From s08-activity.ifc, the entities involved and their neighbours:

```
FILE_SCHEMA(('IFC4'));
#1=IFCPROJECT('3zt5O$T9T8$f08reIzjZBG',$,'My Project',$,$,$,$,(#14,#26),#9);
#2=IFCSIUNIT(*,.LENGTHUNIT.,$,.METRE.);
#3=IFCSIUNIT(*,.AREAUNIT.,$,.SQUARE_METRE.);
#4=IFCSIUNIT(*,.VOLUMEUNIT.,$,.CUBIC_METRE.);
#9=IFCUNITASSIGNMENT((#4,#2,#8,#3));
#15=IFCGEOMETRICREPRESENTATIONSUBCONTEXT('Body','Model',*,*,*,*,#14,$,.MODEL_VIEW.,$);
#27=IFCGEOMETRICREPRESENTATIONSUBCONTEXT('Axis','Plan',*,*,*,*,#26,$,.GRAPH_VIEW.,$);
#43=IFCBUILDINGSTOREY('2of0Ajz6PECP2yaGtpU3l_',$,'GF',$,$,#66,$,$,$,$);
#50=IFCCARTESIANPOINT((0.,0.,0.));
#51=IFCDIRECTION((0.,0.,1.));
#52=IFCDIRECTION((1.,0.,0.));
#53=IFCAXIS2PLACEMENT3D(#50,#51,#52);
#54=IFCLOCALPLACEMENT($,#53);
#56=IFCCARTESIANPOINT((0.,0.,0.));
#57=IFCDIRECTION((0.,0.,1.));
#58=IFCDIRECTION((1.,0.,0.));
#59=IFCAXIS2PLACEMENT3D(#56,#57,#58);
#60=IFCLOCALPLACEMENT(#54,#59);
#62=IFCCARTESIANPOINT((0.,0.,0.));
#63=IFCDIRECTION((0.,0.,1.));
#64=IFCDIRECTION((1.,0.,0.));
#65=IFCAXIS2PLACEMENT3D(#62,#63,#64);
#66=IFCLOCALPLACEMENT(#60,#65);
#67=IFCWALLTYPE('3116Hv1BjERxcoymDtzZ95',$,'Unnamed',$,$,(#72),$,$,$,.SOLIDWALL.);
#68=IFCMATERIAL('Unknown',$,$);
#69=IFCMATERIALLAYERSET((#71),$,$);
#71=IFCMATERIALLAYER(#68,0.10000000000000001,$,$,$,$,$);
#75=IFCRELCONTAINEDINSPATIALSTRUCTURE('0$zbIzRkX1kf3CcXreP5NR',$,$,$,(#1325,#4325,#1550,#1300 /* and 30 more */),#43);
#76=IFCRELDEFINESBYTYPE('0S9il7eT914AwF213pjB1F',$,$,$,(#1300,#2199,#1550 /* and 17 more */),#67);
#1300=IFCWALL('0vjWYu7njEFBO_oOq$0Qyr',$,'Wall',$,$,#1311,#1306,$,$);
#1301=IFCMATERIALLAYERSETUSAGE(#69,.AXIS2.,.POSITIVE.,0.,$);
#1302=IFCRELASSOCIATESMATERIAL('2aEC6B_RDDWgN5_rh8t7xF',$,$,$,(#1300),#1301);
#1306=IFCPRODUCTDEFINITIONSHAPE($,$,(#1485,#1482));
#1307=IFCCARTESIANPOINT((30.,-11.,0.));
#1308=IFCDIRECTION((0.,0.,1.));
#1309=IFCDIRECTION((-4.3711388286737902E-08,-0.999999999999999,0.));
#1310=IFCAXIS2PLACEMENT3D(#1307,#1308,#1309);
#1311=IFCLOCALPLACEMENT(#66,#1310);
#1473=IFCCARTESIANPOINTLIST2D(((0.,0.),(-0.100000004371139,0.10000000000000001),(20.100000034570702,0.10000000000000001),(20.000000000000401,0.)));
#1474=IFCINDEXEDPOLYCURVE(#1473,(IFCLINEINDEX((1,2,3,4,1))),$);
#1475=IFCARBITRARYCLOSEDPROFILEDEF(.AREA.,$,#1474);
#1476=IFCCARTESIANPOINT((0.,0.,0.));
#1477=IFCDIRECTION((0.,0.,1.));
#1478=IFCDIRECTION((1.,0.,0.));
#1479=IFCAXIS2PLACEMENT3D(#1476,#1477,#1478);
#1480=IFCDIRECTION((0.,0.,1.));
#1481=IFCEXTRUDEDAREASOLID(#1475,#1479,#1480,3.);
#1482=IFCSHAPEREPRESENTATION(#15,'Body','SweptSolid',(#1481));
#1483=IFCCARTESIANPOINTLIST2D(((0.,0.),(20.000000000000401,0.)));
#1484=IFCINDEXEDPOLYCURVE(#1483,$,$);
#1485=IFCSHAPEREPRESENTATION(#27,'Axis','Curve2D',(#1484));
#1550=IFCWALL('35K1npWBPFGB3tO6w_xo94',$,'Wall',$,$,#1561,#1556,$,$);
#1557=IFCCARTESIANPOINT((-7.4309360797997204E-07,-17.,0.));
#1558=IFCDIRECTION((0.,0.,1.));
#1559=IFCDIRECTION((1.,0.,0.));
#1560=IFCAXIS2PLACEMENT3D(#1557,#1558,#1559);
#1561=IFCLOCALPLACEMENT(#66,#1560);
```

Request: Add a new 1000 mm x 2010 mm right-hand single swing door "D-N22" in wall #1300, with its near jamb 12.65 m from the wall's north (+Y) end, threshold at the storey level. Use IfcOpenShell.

```python
import numpy as np
import ifcopenshell
import ifcopenshell.api.feature
import ifcopenshell.api.geometry
import ifcopenshell.api.root
import ifcopenshell.api.spatial
import ifcopenshell.geom
import ifcopenshell.util.element
import ifcopenshell.util.placement
import ifcopenshell.util.representation
import ifcopenshell.util.shape
import ifcopenshell.util.unit

model = ifcopenshell.open("s08-activity.ifc")
unit_scale = ifcopenshell.util.unit.calculate_unit_scale(model)
settings = ifcopenshell.geom.settings()


def volume(element):
    """Net volume in cubic metres, openings subtracted."""
    shape = ifcopenshell.geom.create_shape(settings, element)
    return ifcopenshell.util.shape.get_volume(shape.geometry)


wall = model.by_guid("0vjWYu7njEFBO_oOq$0Qyr")
storey = ifcopenshell.util.element.get_container(wall, ifc_class="IfcBuildingStorey")
context = ifcopenshell.util.representation.get_context(model, "Model", "Body", "MODEL_VIEW")
before = volume(wall)

width, height, from_end, sill = 1, 2.01, 12.65, 0.0  # metres

# The wall runs along its own X axis, and the end named is its -X end.
wall_shape = ifcopenshell.geom.create_shape(settings, wall)
x, y, z = ifcopenshell.util.shape.get_vertices(wall_shape.geometry).T
start = x.min() + from_end
face, thickness = float(y.min()), float(y.max() - y.min())
wall_matrix = ifcopenshell.util.placement.get_local_placement(wall.ObjectPlacement)
level = ifcopenshell.util.placement.get_local_placement(storey.ObjectPlacement)[2, 3]


def in_wall(x, y):
    """Placement at x, y metres in the wall's axes, at sill height."""
    matrix = wall_matrix.copy()
    matrix[:, 3] = wall_matrix @ np.array([x / unit_scale, y / unit_scale, 0.0, 1.0])
    matrix[2, 3] = level + sill / unit_scale
    return matrix


# Opening: a box that overshoots both wall faces by 50 mm.
opening = ifcopenshell.api.root.create_entity(model, ifc_class="IfcOpeningElement", predefined_type="OPENING")
box = ifcopenshell.api.geometry.add_wall_representation(
    model, context=context, length=width, height=height, thickness=thickness + 0.1
)
ifcopenshell.api.geometry.assign_representation(model, product=opening, representation=box)
ifcopenshell.api.geometry.edit_object_placement(model, product=opening, matrix=in_wall(start, face - 0.05), is_si=False)
ifcopenshell.api.feature.add_feature(model, feature=opening, element=wall)

door = ifcopenshell.api.root.create_entity(model, ifc_class="IfcDoor", name="D-N22", predefined_type="DOOR")
door.OverallWidth, door.OverallHeight = width / unit_scale, height / unit_scale
door.OperationType = "SINGLE_SWING_RIGHT"
body = ifcopenshell.api.geometry.add_door_representation(
    model,
    context=context,
    overall_width=door.OverallWidth,
    overall_height=door.OverallHeight,
    operation_type="SINGLE_SWING_RIGHT",
    lining_properties={"LiningDepth": thickness / unit_scale, "ThresholdDepth": thickness / unit_scale},
)
ifcopenshell.api.geometry.assign_representation(model, product=door, representation=body)
ifcopenshell.api.spatial.assign_container(model, products=[door], relating_structure=storey)
ifcopenshell.api.feature.add_filling(model, opening=opening, element=door)

# The lining spans the wall, so the door starts at the wall face.
ifcopenshell.api.geometry.edit_object_placement(model, product=door, matrix=in_wall(start, face), is_si=False)

after = volume(wall)

print(f"wall volume {before:.3f} -> {after:.3f} m3")

model.write("s08-activity_updated.ifc")
```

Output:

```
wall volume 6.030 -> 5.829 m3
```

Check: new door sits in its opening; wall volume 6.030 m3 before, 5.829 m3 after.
